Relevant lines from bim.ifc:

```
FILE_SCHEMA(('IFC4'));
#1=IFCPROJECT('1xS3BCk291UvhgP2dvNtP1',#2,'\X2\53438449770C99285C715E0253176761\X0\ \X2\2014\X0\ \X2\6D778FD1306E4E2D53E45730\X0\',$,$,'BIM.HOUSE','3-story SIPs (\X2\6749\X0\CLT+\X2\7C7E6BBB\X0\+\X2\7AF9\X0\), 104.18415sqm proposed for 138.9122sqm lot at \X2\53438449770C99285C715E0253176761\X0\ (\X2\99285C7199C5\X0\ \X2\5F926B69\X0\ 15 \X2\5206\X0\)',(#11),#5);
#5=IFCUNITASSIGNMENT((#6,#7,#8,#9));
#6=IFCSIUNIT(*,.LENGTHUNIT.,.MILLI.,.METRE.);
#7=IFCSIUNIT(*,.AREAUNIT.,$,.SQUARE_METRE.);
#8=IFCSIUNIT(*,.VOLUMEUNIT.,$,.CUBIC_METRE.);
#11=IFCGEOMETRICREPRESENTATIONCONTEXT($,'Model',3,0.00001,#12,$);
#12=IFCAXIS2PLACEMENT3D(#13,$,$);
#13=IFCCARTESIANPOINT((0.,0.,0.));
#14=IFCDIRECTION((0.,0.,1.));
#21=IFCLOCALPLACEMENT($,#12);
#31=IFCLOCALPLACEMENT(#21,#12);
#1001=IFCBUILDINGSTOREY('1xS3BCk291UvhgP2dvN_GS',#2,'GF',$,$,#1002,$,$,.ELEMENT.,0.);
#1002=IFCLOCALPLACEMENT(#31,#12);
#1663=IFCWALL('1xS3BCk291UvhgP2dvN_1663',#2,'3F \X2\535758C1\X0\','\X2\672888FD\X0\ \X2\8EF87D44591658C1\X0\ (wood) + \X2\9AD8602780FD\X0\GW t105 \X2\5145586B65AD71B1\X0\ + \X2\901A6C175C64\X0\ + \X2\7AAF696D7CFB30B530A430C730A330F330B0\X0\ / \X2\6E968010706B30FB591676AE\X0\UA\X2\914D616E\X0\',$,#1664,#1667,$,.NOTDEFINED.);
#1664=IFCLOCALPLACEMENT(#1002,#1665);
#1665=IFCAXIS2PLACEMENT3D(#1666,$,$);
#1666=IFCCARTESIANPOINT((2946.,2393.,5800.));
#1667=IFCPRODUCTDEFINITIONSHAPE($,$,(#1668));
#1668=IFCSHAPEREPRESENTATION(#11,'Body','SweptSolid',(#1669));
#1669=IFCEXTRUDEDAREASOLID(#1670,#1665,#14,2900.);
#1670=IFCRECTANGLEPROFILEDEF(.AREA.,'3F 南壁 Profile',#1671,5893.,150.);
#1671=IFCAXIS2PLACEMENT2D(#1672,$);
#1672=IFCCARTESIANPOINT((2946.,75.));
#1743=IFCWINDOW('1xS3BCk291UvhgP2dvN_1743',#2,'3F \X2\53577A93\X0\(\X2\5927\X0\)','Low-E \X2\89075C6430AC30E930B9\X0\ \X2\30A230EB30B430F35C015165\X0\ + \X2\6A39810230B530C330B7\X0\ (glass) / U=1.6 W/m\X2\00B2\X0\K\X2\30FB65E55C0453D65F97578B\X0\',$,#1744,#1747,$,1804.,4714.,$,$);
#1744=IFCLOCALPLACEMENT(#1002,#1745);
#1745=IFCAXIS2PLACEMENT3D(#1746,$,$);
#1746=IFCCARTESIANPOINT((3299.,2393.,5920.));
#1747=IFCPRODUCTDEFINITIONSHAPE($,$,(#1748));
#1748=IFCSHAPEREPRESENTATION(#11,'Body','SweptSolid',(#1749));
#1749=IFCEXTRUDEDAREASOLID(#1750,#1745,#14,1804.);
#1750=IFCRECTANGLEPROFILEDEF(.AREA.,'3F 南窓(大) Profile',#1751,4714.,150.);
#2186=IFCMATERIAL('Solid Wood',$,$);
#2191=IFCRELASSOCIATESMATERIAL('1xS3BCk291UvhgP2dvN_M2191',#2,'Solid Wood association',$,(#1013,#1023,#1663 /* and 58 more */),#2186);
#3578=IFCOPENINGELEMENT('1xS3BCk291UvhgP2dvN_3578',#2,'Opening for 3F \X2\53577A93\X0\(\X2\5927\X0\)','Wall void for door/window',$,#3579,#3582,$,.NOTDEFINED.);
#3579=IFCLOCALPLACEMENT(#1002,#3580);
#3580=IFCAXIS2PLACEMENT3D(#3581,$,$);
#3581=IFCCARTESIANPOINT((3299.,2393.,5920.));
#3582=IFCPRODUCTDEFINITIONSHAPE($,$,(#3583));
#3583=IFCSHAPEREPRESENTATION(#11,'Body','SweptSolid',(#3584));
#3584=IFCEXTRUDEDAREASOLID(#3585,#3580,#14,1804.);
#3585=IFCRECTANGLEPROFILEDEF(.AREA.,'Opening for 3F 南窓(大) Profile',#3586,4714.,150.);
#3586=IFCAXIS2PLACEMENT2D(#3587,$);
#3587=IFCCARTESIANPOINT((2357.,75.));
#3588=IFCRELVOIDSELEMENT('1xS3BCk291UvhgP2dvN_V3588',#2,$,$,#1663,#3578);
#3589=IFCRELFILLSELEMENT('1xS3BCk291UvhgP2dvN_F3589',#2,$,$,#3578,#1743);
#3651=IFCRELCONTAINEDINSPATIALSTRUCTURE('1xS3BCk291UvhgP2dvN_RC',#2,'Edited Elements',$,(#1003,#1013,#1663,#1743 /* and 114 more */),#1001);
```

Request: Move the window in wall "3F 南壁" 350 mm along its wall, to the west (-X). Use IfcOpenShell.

```python
import ifcopenshell
import ifcopenshell.api.geometry
import ifcopenshell.util.placement
import ifcopenshell.util.unit

model = ifcopenshell.open("bim.ifc")
unit_scale = ifcopenshell.util.unit.calculate_unit_scale(model)

window = model.by_guid("1xS3BCk291UvhgP2dvN_1743")
opening = window.FillsVoids[0].RelatingOpeningElement
wall = opening.VoidsElements[0].RelatingBuildingElement

wall_matrix = ifcopenshell.util.placement.get_local_placement(wall.ObjectPlacement)
shift = wall_matrix[:3, 0] * -0.35 / unit_scale
before = ifcopenshell.util.placement.get_local_placement(window.ObjectPlacement)[:3, 3].copy()

# The window is not placed relative to its opening, so move both.
for product in (opening, window):
    matrix = ifcopenshell.util.placement.get_local_placement(product.ObjectPlacement)
    matrix[:3, 3] += shift
    ifcopenshell.api.geometry.edit_object_placement(model, product=product, matrix=matrix, is_si=False)

after = ifcopenshell.util.placement.get_local_placement(window.ObjectPlacement)[:3, 3]
print("window moved by", (after - before).round(3) + 0.0)

model.write("bim_edited.ifc")
```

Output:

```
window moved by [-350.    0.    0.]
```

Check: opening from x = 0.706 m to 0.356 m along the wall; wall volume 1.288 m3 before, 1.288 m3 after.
